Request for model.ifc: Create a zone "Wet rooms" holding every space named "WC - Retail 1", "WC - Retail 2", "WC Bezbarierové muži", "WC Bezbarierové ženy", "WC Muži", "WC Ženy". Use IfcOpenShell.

First a look at what the model holds.

```python
import ifcopenshell

model = ifcopenshell.open("model.ifc")
print(model.schema)
seen = {}
for space in model.by_type("IfcSpace"):
    seen[space.LongName] = seen.get(space.LongName, 0) + 1
for name, count in sorted(seen.items(), key=str):
    print(count, "x", name)
print("zones:", [z.Name for z in model.by_type("IfcZone")][:20])
```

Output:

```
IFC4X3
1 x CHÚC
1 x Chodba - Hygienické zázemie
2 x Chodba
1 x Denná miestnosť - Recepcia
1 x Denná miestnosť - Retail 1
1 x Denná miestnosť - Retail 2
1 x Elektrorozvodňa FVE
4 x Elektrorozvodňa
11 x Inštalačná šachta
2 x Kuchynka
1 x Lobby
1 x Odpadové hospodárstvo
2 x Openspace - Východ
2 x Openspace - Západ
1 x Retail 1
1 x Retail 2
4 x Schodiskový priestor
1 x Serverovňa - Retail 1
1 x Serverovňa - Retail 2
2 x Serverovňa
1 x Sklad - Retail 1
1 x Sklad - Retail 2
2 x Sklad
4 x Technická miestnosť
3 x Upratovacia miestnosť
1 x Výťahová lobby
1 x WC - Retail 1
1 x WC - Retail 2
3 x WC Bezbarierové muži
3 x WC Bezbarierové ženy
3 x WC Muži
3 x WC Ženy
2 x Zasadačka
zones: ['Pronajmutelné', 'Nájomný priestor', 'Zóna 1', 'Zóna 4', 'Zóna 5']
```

```python
import ifcopenshell
import ifcopenshell.api.group
import ifcopenshell.api.root

model = ifcopenshell.open("model.ifc")

names = {"WC - Retail 1", "WC - Retail 2", "WC Bezbarierové muži", "WC Bezbarierové ženy", "WC Muži", "WC Ženy"}
spaces = [s for s in model.by_type("IfcSpace") if s.LongName in names]

zone = ifcopenshell.api.root.create_entity(model, ifc_class="IfcZone", name="Wet rooms")
ifcopenshell.api.group.assign_group(model, products=spaces, group=zone)
print(len(spaces), "spaces in", zone.Name)

model.write("model-out.ifc")
```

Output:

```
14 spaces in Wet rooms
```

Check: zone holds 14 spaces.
